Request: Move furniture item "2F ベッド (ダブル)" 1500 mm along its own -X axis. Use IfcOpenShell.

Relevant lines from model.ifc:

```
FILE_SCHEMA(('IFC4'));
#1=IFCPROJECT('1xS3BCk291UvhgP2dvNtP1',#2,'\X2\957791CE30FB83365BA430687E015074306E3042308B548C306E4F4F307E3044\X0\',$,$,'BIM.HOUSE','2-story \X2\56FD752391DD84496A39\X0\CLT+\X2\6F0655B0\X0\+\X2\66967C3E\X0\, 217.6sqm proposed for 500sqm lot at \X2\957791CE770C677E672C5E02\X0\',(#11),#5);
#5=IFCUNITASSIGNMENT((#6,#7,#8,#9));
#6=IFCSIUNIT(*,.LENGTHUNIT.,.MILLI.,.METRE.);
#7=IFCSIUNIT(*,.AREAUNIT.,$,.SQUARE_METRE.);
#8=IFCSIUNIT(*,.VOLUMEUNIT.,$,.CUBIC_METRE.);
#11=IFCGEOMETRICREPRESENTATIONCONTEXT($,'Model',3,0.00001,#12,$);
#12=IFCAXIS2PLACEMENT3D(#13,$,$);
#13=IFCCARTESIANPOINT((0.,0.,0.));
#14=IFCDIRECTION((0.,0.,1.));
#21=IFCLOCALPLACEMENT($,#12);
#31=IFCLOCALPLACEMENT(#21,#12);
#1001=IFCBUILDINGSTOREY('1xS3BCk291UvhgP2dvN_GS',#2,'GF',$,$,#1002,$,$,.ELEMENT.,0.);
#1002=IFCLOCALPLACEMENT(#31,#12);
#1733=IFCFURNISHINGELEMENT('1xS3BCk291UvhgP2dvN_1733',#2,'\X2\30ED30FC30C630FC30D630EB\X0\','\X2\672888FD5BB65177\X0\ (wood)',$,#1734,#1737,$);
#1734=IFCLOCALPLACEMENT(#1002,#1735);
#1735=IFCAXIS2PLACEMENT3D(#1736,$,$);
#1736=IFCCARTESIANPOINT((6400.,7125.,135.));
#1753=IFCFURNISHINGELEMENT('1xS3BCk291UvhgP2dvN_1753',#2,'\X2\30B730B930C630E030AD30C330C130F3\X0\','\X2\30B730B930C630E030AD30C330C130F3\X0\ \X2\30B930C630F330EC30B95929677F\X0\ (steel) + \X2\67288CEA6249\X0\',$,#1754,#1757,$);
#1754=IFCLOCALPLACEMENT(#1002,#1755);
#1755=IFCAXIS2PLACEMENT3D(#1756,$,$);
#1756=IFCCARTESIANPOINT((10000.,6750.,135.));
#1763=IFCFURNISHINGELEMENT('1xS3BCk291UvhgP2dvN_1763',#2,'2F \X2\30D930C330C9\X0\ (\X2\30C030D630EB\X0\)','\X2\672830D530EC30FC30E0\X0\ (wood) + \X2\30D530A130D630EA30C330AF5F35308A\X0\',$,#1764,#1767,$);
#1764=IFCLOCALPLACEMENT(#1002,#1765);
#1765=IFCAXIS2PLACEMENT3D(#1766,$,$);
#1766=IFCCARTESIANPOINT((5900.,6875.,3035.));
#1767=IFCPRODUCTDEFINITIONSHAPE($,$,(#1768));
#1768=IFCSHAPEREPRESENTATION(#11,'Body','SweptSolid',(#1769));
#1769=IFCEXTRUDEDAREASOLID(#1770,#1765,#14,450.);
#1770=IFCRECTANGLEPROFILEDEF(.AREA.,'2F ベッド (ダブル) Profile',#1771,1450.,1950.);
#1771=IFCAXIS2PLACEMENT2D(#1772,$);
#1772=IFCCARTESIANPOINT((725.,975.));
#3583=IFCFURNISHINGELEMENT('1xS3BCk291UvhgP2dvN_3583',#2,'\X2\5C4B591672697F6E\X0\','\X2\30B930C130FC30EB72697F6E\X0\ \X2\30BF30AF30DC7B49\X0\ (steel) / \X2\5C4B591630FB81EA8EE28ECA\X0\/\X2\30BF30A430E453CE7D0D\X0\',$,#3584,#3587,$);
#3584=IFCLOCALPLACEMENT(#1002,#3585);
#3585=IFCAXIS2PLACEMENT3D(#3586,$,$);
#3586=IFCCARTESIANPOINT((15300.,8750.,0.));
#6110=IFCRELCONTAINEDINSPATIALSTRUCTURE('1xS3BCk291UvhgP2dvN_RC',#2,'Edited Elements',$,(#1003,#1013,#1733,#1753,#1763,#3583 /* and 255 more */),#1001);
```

```python
import ifcopenshell
import ifcopenshell.api.geometry
import ifcopenshell.util.placement
import ifcopenshell.util.unit

model = ifcopenshell.open("model.ifc")
unit_scale = ifcopenshell.util.unit.calculate_unit_scale(model)

item = model.by_guid("1xS3BCk291UvhgP2dvN_1763")
matrix = ifcopenshell.util.placement.get_local_placement(item.ObjectPlacement)
matrix[:3, 3] -= matrix[:3, 0] * 1.5 / unit_scale
ifcopenshell.api.geometry.edit_object_placement(model, product=item, matrix=matrix, is_si=False)

print(ifcopenshell.util.placement.get_local_placement(item.ObjectPlacement).round(3) + 0.0)

model.write("model_rev.ifc")
```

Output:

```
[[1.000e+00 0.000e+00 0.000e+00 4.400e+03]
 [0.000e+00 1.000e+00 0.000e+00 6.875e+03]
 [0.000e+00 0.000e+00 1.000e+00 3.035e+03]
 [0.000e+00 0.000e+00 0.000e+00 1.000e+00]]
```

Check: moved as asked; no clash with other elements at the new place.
